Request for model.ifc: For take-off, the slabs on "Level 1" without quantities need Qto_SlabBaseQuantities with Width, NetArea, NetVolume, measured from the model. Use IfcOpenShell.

First a look at what the model holds.

```python
import ifcopenshell
import ifcopenshell.util.element
import ifcopenshell.util.unit

model = ifcopenshell.open("model.ifc")
print(model.schema)
for unit_type in ("LENGTHUNIT", "AREAUNIT", "VOLUMEUNIT"):
    print(unit_type, ifcopenshell.util.unit.calculate_unit_scale(model, unit_type))
storey = next(s for s in model.by_type("IfcBuildingStorey") if s.Name == "Level 1")
slabs = [e for e in ifcopenshell.util.element.get_decomposition(storey) if e.is_a("IfcSlab")]
for e in sorted(slabs, key=lambda e: e.id()):
    print(e.id(), e.is_a(), e.Name, list(ifcopenshell.util.element.get_psets(e, qtos_only=True)), sep=" | ")
```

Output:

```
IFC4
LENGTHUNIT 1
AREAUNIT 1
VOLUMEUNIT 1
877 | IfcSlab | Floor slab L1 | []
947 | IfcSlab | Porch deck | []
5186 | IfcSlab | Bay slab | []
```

```python
import ifcopenshell
import ifcopenshell.api.pset
import ifcopenshell.geom
import ifcopenshell.util.element
import ifcopenshell.util.shape
import ifcopenshell.util.unit

model = ifcopenshell.open("model.ifc")
unit_scale = ifcopenshell.util.unit.calculate_unit_scale(model)
area_scale = ifcopenshell.util.unit.calculate_unit_scale(model, "AREAUNIT")
volume_scale = ifcopenshell.util.unit.calculate_unit_scale(model, "VOLUMEUNIT")
settings = ifcopenshell.geom.settings()

storey = next(s for s in model.by_type("IfcBuildingStorey") if s.Name == "Level 1")
slabs = [e for e in ifcopenshell.util.element.get_decomposition(storey) if e.is_a("IfcSlab")]

for e in sorted(slabs, key=lambda e: e.id()):
    if ifcopenshell.util.element.get_psets(e, qtos_only=True, should_inherit=False):
        continue
    # Geometry comes back in metres, in the element's own axes.
    shape = ifcopenshell.geom.create_shape(settings, e)
    values = {
        "Width": ifcopenshell.util.shape.get_z(shape.geometry) / unit_scale,
        "NetArea": ifcopenshell.util.shape.get_footprint_area(shape.geometry) / area_scale,
        "NetVolume": ifcopenshell.util.shape.get_volume(shape.geometry) / volume_scale,
    }
    qto = ifcopenshell.api.pset.add_qto(model, product=e, name="Qto_SlabBaseQuantities")
    ifcopenshell.api.pset.edit_qto(model, qto=qto, properties=values)
    print(e.id(), {k: round(v, 3) for k, v in values.items()})

model.write("model_rev.ifc")
```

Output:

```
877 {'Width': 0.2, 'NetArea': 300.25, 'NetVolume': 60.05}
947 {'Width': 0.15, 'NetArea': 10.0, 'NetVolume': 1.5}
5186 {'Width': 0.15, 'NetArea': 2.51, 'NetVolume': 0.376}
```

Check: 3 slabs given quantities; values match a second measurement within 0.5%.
